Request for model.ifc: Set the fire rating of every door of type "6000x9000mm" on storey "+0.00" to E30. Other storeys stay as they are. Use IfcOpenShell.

First a look at what the model holds.

```python
import ifcopenshell
import ifcopenshell.util.element

model = ifcopenshell.open("model.ifc")
print(model.schema)
storey = next(s for s in model.by_type("IfcBuildingStorey") if s.Name == "+0.00")
doors = [e for e in ifcopenshell.util.element.get_decomposition(storey) if e.is_a("IfcDoor")]
seen = {}
for e in doors:
    element_type = ifcopenshell.util.element.get_type(e)
    key = (element_type.Name if element_type != e and element_type else None, ifcopenshell.util.element.get_pset(e, "Pset_DoorCommon", "FireRating"))
    seen[key] = seen.get(key, 0) + 1
for (name, value), count in sorted(seen.items(), key=str):
    print(count, "x", name, "|", value)
```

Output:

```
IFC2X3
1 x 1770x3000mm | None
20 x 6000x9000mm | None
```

```python
import ifcopenshell
import ifcopenshell.api.pset
import ifcopenshell.util.element

model = ifcopenshell.open("model.ifc")

storey = next(s for s in model.by_type("IfcBuildingStorey") if s.Name == "+0.00")
doors = [e for e in ifcopenshell.util.element.get_decomposition(storey) if e.is_a("IfcDoor")]

count = 0
for e in doors:
    element_type = ifcopenshell.util.element.get_type(e)
    if element_type in (None, e) or element_type.Name != "6000x9000mm":
        continue
    # add_pset returns the element's existing set when there is one.
    pset = ifcopenshell.api.pset.add_pset(model, product=e, name="Pset_DoorCommon")
    ifcopenshell.api.pset.edit_pset(model, pset=pset, properties={"FireRating": "E30"})
    count += 1

print(count, "doors updated")

model.write("model_rev.ifc")
```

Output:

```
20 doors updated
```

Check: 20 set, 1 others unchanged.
